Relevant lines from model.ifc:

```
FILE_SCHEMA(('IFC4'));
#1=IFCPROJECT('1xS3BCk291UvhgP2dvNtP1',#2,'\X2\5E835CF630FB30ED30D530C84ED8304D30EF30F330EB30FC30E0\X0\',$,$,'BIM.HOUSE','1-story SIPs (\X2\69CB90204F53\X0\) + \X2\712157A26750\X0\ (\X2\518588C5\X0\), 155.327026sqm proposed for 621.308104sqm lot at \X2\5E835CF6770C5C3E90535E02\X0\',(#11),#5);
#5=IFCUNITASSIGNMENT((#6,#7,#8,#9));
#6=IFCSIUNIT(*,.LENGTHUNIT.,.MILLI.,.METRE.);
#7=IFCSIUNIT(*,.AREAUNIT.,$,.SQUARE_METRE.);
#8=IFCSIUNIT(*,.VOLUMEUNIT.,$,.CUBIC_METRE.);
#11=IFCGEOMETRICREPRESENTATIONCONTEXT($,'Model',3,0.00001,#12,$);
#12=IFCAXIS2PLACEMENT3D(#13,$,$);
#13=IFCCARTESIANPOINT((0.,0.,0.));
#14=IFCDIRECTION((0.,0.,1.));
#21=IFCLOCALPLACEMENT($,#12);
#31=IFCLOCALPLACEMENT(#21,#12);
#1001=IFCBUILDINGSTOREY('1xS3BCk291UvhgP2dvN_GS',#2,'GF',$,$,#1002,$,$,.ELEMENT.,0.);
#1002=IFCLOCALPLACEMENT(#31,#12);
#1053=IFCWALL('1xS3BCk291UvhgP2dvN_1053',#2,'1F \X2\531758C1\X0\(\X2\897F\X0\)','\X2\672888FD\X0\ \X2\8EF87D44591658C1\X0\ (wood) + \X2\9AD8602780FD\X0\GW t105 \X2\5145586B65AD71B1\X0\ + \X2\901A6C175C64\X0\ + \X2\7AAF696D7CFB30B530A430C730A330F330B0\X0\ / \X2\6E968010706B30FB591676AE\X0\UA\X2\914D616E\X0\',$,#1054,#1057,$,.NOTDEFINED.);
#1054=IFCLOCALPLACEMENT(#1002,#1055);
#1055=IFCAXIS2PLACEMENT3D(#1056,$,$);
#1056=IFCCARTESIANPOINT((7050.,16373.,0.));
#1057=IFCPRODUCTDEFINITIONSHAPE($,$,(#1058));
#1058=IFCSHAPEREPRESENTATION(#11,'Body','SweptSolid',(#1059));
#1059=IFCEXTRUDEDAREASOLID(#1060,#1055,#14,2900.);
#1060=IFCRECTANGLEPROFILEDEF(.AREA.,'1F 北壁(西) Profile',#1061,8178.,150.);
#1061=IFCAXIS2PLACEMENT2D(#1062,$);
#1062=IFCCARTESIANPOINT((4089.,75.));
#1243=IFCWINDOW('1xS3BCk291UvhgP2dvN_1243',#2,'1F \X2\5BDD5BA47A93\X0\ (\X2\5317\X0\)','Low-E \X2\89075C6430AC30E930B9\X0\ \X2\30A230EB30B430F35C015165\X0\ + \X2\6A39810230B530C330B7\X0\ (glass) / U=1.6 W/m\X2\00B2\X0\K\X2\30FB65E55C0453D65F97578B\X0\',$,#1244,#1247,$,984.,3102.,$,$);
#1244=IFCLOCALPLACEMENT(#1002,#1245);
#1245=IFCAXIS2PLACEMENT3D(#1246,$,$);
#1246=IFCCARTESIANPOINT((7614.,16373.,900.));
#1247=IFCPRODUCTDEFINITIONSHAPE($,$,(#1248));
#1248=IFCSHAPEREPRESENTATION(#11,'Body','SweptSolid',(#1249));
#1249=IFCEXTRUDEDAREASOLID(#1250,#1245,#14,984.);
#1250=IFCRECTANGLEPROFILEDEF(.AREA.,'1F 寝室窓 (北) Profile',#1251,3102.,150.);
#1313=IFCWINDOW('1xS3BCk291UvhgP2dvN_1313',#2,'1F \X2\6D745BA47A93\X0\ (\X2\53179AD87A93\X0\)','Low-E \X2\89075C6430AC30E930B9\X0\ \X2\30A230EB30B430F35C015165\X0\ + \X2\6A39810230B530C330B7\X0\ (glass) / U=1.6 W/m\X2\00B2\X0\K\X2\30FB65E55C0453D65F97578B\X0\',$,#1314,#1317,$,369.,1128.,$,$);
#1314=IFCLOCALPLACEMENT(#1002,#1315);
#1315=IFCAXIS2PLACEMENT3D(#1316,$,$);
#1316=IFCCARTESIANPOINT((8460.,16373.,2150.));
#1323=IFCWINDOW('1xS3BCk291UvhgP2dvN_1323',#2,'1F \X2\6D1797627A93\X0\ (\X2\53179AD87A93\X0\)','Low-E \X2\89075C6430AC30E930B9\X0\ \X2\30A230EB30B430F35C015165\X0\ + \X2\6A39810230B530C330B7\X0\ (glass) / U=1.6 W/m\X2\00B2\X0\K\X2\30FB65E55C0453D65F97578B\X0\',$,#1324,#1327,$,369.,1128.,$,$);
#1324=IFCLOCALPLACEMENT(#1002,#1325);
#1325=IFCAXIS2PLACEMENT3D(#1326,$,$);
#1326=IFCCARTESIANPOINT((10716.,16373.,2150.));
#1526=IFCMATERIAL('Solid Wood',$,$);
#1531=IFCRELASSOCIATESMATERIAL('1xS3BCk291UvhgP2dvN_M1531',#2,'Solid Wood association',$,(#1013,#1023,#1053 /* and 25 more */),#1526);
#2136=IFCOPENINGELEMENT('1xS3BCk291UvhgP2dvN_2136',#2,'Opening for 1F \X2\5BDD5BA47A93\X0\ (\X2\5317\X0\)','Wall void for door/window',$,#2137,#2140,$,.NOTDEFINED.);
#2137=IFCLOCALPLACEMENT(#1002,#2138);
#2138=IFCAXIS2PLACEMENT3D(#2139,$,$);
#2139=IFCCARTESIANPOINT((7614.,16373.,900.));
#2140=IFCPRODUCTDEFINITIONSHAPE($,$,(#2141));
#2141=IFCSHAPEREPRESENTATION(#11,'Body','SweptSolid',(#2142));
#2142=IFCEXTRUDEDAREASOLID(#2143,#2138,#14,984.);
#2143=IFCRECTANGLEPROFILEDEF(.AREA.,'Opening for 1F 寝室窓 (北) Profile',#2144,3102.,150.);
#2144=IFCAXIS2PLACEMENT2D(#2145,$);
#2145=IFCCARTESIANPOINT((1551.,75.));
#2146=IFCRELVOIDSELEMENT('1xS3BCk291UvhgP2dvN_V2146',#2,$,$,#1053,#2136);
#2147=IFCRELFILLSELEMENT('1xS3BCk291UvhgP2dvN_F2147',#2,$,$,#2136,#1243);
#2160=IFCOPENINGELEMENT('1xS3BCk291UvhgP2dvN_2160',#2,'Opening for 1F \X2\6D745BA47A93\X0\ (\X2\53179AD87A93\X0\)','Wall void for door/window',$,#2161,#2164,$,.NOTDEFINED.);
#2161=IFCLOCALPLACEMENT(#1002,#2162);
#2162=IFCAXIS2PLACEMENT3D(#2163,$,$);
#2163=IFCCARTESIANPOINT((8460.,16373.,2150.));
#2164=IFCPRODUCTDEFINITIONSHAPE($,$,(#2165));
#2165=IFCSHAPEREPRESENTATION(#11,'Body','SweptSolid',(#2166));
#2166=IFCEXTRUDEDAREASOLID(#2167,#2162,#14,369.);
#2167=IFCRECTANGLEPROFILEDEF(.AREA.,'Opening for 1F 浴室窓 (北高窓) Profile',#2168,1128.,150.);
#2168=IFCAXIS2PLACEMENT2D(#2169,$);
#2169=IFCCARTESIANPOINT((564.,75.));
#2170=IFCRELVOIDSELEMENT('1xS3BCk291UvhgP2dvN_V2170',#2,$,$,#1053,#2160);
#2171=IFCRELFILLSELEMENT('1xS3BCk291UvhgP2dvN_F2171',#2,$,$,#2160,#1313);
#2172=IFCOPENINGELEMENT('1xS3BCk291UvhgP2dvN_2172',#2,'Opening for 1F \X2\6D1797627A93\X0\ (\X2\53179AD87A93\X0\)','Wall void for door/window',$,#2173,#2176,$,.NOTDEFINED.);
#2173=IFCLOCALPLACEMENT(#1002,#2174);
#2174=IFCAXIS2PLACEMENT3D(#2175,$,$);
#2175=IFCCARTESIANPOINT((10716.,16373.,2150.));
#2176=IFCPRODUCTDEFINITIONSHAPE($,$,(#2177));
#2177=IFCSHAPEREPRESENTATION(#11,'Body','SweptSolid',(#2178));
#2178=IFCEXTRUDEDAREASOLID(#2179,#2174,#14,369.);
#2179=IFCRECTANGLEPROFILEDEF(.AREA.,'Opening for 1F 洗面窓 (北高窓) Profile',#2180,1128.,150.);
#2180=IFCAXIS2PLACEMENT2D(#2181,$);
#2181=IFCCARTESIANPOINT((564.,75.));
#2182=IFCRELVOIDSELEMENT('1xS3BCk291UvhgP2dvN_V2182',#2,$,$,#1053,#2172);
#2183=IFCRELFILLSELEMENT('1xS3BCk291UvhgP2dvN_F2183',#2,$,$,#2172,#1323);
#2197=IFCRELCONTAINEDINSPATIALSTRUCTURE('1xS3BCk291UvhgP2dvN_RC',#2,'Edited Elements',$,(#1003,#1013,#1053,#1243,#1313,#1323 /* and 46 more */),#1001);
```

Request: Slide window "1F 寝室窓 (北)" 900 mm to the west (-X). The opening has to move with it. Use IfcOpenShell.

```python
import ifcopenshell
import ifcopenshell.api.geometry
import ifcopenshell.util.placement

model = ifcopenshell.open("model.ifc")

window = model.by_guid("1xS3BCk291UvhgP2dvN_1243")
opening = window.FillsVoids[0].RelatingOpeningElement
wall = opening.VoidsElements[0].RelatingBuildingElement

wall_matrix = ifcopenshell.util.placement.get_local_placement(wall.ObjectPlacement)
shift = wall_matrix[:3, 0] * -900.0
before = ifcopenshell.util.placement.get_local_placement(window.ObjectPlacement)[:3, 3].copy()

# The window is not placed relative to its opening, so move both.
for product in (opening, window):
    matrix = ifcopenshell.util.placement.get_local_placement(product.ObjectPlacement)
    matrix[:3, 3] += shift
    ifcopenshell.api.geometry.edit_object_placement(model, product=product, matrix=matrix, is_si=False)

after = ifcopenshell.util.placement.get_local_placement(window.ObjectPlacement)[:3, 3]
print("window moved by", (after - before).round(3) + 0.0)

model.write("model_v2.ifc")
```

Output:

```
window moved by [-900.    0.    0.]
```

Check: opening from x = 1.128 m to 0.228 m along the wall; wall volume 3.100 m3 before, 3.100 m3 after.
